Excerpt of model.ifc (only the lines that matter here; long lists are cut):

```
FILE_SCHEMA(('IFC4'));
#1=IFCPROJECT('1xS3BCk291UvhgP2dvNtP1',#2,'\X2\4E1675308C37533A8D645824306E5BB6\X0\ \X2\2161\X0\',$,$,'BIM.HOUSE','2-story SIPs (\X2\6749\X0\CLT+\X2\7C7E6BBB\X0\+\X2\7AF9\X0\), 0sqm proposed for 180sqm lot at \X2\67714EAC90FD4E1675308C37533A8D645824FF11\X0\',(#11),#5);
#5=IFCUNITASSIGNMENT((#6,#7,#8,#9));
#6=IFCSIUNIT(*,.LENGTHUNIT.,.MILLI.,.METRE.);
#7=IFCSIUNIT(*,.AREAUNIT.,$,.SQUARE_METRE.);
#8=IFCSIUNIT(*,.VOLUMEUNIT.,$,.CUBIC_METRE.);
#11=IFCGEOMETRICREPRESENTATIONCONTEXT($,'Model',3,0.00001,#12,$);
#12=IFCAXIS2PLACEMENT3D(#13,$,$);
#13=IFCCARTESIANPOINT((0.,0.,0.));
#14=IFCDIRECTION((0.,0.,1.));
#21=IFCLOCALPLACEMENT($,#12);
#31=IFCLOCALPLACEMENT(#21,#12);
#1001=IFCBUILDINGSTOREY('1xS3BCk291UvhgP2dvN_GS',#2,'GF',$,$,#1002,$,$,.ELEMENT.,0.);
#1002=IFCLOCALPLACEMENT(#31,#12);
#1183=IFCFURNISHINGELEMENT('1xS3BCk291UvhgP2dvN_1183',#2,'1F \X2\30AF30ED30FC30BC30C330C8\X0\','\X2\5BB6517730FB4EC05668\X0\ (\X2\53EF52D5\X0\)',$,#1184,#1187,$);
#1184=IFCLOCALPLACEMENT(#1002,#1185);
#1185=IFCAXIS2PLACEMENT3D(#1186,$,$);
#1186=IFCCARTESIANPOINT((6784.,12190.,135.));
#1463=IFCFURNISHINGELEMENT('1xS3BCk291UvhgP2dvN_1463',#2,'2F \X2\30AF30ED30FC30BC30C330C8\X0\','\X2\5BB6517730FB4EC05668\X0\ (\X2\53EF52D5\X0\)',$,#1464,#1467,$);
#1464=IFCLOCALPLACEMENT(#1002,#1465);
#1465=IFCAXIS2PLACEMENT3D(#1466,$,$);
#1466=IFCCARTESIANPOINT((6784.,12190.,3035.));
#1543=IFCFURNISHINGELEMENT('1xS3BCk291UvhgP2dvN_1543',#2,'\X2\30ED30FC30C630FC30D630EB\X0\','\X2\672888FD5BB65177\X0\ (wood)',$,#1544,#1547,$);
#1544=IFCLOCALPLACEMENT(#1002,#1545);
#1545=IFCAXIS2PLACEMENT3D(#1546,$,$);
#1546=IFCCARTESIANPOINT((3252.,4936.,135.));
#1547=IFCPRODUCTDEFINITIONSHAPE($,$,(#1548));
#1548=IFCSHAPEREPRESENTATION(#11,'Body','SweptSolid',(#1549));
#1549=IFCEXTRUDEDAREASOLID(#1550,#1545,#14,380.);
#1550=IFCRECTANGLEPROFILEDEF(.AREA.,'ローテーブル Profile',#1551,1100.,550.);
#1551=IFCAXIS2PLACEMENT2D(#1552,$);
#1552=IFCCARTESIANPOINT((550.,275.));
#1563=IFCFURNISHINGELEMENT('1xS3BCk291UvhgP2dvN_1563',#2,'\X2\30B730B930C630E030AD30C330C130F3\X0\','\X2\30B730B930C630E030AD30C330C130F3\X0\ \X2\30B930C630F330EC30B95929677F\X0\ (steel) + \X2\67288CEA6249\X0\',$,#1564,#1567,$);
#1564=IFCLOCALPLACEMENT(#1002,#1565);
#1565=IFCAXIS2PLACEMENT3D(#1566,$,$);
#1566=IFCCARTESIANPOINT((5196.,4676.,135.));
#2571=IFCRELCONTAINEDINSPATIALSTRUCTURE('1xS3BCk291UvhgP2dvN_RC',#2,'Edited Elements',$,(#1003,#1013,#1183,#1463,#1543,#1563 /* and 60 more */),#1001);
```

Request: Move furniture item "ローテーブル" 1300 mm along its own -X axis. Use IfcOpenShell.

```python
import ifcopenshell
import ifcopenshell.api.geometry
import ifcopenshell.util.placement
import ifcopenshell.util.unit

model = ifcopenshell.open("model.ifc")
unit_scale = ifcopenshell.util.unit.calculate_unit_scale(model)

item = model.by_guid("1xS3BCk291UvhgP2dvN_1543")
matrix = ifcopenshell.util.placement.get_local_placement(item.ObjectPlacement)
matrix[:3, 3] -= matrix[:3, 0] * 1.3 / unit_scale
ifcopenshell.api.geometry.edit_object_placement(model, product=item, matrix=matrix, is_si=False)

print(ifcopenshell.util.placement.get_local_placement(item.ObjectPlacement).round(3) + 0.0)

model.write("model_updated.ifc")
```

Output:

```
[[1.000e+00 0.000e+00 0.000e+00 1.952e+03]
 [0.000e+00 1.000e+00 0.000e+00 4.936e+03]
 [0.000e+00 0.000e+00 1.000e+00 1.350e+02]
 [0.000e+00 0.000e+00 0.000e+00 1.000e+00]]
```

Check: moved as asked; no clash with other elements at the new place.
